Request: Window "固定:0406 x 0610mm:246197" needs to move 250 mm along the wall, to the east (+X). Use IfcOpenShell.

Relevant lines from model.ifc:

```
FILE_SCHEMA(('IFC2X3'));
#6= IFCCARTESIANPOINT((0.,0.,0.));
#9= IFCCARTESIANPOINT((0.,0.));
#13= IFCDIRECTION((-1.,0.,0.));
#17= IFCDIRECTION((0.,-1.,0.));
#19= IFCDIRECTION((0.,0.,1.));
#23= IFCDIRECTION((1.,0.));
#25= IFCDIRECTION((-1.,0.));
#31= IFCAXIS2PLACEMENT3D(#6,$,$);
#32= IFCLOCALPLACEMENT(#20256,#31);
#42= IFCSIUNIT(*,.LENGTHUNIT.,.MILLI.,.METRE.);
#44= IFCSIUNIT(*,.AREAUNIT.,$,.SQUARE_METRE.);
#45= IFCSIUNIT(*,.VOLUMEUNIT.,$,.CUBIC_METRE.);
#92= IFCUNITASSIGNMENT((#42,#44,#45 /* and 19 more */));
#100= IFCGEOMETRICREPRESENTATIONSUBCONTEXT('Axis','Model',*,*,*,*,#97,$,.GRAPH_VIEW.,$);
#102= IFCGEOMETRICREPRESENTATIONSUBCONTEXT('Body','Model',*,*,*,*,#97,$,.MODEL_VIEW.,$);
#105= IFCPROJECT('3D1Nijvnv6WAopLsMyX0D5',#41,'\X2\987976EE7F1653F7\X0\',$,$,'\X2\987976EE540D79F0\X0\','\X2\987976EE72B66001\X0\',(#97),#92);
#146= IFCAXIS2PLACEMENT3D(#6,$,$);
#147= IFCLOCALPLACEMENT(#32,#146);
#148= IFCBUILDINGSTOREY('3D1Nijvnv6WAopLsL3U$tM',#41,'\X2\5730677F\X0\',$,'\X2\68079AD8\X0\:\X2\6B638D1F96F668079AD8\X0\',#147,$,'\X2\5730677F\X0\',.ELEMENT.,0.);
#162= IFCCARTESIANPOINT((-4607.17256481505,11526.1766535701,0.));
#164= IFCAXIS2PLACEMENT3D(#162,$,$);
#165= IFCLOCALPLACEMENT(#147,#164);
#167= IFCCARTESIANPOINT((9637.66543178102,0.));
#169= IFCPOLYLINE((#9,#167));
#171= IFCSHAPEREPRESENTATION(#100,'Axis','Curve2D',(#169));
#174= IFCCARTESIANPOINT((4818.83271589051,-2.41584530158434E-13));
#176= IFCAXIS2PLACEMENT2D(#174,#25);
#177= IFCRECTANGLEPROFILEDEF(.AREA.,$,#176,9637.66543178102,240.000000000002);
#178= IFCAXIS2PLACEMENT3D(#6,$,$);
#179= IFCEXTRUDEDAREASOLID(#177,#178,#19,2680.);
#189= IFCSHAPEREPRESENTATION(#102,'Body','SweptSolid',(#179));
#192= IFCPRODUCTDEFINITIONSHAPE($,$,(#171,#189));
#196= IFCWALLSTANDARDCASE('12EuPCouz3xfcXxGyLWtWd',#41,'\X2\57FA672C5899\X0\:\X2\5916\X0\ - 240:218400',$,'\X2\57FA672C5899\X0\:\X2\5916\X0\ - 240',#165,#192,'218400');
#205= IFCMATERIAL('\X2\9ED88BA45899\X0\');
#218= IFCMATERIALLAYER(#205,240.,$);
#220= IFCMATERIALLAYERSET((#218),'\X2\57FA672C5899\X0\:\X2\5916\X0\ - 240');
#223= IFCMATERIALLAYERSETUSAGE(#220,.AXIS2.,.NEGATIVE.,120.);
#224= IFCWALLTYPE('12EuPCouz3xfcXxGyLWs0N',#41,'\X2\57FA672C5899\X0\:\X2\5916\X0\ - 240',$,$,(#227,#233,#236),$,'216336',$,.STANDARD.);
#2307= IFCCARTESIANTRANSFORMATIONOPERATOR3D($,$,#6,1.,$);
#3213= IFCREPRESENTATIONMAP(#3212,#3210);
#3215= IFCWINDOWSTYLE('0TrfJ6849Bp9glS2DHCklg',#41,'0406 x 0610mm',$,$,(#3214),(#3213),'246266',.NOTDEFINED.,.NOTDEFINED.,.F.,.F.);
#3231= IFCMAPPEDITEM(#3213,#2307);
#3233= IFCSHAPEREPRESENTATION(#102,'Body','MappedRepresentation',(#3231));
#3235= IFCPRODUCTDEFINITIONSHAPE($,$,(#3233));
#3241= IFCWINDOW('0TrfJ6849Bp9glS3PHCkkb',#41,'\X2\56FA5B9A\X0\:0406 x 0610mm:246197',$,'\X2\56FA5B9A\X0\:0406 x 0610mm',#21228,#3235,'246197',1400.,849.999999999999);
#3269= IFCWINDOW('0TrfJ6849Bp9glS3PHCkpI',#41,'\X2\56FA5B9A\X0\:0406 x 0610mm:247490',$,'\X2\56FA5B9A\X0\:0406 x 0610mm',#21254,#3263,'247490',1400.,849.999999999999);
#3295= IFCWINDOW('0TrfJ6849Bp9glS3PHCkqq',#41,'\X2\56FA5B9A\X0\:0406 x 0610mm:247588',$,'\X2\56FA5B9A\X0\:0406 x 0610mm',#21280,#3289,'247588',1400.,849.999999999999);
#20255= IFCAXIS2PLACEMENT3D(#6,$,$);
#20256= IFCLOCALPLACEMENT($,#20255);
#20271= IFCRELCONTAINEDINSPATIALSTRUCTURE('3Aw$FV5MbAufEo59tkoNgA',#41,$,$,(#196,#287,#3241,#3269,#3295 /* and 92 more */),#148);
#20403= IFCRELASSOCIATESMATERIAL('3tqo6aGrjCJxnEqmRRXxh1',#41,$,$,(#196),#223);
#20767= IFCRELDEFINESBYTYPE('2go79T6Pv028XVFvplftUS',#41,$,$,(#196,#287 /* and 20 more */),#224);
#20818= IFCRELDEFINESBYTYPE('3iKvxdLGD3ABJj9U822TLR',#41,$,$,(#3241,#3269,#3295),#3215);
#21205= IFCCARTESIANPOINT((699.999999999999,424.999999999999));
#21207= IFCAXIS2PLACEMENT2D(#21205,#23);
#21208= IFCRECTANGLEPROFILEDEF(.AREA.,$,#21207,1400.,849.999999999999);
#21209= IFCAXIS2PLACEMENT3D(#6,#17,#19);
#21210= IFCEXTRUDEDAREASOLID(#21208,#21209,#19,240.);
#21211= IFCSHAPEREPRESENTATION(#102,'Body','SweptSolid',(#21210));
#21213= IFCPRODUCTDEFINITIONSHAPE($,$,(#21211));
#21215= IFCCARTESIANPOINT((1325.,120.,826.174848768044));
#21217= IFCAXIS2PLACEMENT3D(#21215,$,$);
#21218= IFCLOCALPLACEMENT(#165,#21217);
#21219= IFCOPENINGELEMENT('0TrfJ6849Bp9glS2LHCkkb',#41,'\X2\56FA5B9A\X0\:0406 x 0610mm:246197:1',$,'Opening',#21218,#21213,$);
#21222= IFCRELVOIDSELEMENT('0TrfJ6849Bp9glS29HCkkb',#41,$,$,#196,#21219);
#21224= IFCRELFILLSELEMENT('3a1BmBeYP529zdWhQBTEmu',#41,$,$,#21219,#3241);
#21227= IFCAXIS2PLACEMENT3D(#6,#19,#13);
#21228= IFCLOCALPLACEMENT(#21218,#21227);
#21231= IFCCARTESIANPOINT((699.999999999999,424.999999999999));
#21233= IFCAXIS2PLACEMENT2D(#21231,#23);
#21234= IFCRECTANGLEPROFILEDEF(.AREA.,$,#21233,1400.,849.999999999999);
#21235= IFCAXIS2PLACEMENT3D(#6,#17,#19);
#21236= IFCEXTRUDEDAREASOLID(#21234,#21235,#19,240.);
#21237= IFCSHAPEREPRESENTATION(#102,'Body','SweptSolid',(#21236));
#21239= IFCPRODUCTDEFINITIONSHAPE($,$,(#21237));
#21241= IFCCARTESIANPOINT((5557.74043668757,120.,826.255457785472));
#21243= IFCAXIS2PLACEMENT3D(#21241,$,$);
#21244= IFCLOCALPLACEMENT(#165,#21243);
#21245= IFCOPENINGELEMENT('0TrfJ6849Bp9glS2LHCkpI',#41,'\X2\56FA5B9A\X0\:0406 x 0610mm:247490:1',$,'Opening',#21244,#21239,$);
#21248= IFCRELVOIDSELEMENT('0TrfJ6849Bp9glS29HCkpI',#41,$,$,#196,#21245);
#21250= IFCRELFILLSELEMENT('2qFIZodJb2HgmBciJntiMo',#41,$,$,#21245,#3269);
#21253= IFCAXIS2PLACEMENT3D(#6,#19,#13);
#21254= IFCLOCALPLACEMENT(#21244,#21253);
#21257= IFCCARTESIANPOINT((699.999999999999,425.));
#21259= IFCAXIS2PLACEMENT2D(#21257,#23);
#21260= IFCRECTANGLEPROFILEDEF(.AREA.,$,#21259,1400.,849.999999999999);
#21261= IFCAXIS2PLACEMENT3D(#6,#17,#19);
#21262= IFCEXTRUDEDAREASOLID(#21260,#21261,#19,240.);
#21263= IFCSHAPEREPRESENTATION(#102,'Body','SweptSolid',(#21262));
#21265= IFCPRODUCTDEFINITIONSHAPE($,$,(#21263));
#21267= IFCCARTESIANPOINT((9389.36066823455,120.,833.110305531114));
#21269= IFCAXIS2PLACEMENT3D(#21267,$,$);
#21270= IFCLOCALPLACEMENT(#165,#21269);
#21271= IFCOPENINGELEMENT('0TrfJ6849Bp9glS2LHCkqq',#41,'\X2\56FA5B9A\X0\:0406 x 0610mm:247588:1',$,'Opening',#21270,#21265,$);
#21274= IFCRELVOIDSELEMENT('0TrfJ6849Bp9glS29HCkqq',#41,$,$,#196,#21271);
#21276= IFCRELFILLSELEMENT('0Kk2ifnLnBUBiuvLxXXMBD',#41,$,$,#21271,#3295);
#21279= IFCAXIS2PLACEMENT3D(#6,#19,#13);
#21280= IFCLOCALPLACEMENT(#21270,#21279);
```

```python
import ifcopenshell
import ifcopenshell.api.geometry
import ifcopenshell.util.placement
import ifcopenshell.util.unit

model = ifcopenshell.open("model.ifc")
unit_scale = ifcopenshell.util.unit.calculate_unit_scale(model)

window = model.by_id(3241)
opening = window.FillsVoids[0].RelatingOpeningElement
wall = opening.VoidsElements[0].RelatingBuildingElement

wall_matrix = ifcopenshell.util.placement.get_local_placement(wall.ObjectPlacement)
shift = wall_matrix[:3, 0] * 0.25 / unit_scale
before = ifcopenshell.util.placement.get_local_placement(window.ObjectPlacement)[:3, 3].copy()

# The window is placed relative to its opening, so it follows when the opening moves.
matrix = ifcopenshell.util.placement.get_local_placement(opening.ObjectPlacement)
matrix[:3, 3] += shift
ifcopenshell.api.geometry.edit_object_placement(
    model, product=opening, matrix=matrix, is_si=False, should_transform_children=True
)

after = ifcopenshell.util.placement.get_local_placement(window.ObjectPlacement)[:3, 3]
print("window moved by", (after - before).round(3) + 0.0)

model.write("model_v2.ifc")
```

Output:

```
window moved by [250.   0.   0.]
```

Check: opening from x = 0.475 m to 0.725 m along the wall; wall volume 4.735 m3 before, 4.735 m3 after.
